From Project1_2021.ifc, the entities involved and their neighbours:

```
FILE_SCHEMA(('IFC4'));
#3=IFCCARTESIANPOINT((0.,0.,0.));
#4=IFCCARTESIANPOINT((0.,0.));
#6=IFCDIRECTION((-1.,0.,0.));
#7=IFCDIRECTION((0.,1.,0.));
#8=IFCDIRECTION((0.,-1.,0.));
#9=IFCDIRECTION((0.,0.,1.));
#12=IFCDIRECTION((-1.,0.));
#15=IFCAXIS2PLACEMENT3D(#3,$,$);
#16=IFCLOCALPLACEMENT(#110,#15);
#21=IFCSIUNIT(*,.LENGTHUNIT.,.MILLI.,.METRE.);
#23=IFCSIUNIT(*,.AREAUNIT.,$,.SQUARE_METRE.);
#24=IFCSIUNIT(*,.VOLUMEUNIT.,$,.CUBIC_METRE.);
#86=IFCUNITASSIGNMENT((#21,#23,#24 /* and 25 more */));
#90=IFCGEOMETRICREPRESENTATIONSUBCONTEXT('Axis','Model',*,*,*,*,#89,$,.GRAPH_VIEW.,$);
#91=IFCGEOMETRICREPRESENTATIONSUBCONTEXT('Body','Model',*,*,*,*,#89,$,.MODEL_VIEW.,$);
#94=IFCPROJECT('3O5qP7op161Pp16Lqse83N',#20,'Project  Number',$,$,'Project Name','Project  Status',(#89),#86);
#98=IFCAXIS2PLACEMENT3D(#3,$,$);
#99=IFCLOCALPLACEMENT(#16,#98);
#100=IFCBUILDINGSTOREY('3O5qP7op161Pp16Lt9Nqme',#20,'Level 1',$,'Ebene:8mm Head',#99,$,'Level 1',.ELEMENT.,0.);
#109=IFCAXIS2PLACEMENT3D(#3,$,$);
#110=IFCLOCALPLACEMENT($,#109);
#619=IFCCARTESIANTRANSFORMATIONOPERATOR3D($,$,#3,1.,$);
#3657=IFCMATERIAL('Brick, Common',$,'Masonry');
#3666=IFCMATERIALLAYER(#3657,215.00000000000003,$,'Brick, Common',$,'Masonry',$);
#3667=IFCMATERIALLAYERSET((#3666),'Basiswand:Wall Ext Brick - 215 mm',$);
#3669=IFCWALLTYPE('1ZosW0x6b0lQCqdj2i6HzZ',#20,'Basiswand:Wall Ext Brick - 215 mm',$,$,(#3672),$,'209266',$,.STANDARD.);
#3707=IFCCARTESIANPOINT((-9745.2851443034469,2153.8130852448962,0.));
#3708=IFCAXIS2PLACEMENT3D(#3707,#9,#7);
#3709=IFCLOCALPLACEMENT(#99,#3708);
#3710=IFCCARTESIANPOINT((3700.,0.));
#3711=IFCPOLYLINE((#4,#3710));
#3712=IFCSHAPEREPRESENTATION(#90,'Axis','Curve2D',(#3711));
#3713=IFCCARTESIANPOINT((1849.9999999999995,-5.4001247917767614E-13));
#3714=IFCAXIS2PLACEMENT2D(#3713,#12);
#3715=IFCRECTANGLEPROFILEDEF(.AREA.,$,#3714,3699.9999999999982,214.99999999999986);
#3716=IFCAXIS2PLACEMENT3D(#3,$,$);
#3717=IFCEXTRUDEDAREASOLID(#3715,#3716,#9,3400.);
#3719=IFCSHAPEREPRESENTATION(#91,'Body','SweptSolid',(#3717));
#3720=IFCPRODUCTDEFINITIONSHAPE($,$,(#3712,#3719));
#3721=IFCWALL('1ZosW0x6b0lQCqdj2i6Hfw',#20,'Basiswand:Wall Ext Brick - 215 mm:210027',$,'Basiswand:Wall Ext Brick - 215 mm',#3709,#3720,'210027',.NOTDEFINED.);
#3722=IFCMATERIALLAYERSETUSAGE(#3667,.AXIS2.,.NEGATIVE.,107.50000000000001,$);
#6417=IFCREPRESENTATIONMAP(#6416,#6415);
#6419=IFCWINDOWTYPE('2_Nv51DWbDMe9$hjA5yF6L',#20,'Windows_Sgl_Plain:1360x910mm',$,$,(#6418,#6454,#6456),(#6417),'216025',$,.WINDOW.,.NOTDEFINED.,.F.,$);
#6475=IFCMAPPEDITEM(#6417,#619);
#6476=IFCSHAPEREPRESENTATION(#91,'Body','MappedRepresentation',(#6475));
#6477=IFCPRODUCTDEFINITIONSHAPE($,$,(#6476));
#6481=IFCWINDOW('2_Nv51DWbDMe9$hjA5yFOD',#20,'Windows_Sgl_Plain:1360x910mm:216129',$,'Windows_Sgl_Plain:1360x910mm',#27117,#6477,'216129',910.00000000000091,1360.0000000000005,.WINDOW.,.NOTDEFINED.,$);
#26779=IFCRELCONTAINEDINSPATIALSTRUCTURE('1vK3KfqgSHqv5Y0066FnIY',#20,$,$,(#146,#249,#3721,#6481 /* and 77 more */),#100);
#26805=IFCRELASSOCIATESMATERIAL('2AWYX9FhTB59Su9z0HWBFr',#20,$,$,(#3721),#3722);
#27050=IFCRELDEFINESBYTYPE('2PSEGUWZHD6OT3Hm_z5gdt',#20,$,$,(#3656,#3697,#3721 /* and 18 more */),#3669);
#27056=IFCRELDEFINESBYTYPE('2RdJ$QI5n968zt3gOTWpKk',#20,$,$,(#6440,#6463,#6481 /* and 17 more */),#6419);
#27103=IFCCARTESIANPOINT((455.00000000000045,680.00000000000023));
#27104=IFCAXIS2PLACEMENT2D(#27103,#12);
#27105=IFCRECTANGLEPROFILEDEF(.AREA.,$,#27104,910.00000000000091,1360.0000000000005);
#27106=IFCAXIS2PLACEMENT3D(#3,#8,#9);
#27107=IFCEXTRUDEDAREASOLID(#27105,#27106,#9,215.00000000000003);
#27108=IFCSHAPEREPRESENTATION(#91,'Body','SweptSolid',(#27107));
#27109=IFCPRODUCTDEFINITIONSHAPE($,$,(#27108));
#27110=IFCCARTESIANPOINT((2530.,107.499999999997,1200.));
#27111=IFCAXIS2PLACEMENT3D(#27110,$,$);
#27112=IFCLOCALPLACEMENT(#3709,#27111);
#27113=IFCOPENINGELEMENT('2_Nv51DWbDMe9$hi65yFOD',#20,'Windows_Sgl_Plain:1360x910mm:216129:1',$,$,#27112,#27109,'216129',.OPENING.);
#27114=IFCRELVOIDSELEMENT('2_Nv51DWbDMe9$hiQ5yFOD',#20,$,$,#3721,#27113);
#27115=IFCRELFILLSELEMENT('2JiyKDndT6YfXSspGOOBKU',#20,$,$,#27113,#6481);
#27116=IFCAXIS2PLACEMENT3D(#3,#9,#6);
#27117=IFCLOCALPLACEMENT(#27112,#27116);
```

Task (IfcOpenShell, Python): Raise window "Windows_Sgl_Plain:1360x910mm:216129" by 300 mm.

```python
import numpy as np
import ifcopenshell
import ifcopenshell.api.geometry
import ifcopenshell.util.placement
import ifcopenshell.util.unit

model = ifcopenshell.open("Project1_2021.ifc")
unit_scale = ifcopenshell.util.unit.calculate_unit_scale(model)

window = model.by_guid("2_Nv51DWbDMe9$hjA5yFOD")
opening = window.FillsVoids[0].RelatingOpeningElement
dz = 0.3 / unit_scale

shift = np.array([0.0, 0.0, dz])
# The window is placed relative to its opening, so it follows when the opening moves.
matrix = ifcopenshell.util.placement.get_local_placement(opening.ObjectPlacement)
matrix[:3, 3] += shift
ifcopenshell.api.geometry.edit_object_placement(
    model, product=opening, matrix=matrix, is_si=False, should_transform_children=True
)

print(f"moved by {dz * unit_scale:+.3f} m")

model.write("Project1_2021-out.ifc")
```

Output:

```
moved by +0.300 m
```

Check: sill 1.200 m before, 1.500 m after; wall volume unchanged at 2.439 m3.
